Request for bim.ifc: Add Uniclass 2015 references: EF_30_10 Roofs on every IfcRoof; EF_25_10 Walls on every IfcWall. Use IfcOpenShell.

First a look at what the model holds.

```python
import ifcopenshell

model = ifcopenshell.open("bim.ifc")
print(model.schema)
print("classifications:", [c.Name for c in model.by_type("IfcClassification")])
for ifc_class in ("IfcDoor", "IfcRoof", "IfcStair", "IfcWall", "IfcWindow"):
    print(ifc_class, len(model.by_type(ifc_class)))
```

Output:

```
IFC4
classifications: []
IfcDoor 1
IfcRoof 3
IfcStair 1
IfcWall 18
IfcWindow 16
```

```python
import ifcopenshell
import ifcopenshell.api.classification

model = ifcopenshell.open("bim.ifc")

system = ifcopenshell.api.classification.add_classification(model, classification="Uniclass 2015")

codes = {
    "IfcRoof": ("EF_30_10", "Roofs"),
    "IfcWall": ("EF_25_10", "Walls"),
}
for ifc_class, (code, name) in codes.items():
    products = model.by_type(ifc_class)
    ifcopenshell.api.classification.add_reference(
        model, products=products, classification=system, identification=code, name=name
    )
    print(code, len(products))

model.write("bim_edited.ifc")
```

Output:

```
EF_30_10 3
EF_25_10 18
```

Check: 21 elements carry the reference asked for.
